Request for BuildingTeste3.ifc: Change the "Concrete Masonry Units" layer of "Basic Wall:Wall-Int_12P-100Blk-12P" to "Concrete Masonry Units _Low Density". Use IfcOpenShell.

First a look at what the model holds.

```python
import ifcopenshell
import ifcopenshell.util.element

model = ifcopenshell.open("BuildingTeste3.ifc")
print(model.schema)
for layer_set in model.by_type("IfcMaterialLayerSet"):
    if layer_set.LayerSetName == "Basic Wall:Wall-Int_12P-100Blk-12P":
        for layer in layer_set.MaterialLayers:
            print(layer.id(), layer.Material and layer.Material.Name, layer.LayerThickness, sep=" | ")
        print(len(ifcopenshell.util.element.get_elements_by_material(model, layer_set)), "elements and types use it")
print(sorted(m.Name for m in model.by_type("IfcMaterial") if m.Name)[:60])
```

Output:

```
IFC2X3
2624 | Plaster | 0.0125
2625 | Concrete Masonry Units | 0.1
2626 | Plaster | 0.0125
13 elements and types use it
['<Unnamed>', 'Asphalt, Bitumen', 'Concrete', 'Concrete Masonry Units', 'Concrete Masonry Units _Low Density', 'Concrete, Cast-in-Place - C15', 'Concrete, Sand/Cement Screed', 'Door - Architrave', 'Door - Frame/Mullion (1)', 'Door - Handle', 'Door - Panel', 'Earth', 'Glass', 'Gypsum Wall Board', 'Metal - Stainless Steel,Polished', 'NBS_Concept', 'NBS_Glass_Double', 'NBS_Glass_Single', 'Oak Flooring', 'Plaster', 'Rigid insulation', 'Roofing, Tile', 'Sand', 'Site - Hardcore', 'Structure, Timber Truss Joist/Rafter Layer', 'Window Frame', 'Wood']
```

```python
import ifcopenshell
import ifcopenshell.api.material

model = ifcopenshell.open("BuildingTeste3.ifc")

layer_set = next(s for s in model.by_type("IfcMaterialLayerSet") if s.LayerSetName == "Basic Wall:Wall-Int_12P-100Blk-12P")
layer = next(l for l in layer_set.MaterialLayers if l.Material and l.Material.Name == "Concrete Masonry Units")
material = next(m for m in model.by_type("IfcMaterial") if m.Name == "Concrete Masonry Units _Low Density")

# Point this one layer at the other material; renaming the old one would change it everywhere.
ifcopenshell.api.material.edit_layer(model, layer=layer, attributes={}, material=material)

print([l.Material.Name if l.Material else None for l in layer_set.MaterialLayers])

model.write("BuildingTeste3_rev.ifc")
```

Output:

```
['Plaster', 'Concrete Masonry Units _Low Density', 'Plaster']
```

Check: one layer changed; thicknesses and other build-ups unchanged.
